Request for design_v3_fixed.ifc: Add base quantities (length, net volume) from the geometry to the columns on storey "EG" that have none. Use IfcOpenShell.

First a look at what the model holds.

```python
import ifcopenshell
import ifcopenshell.util.element
import ifcopenshell.util.unit

model = ifcopenshell.open("design_v3_fixed.ifc")
print(model.schema)
for unit_type in ("LENGTHUNIT", "AREAUNIT", "VOLUMEUNIT"):
    print(unit_type, ifcopenshell.util.unit.calculate_unit_scale(model, unit_type))
storey = next(s for s in model.by_type("IfcBuildingStorey") if s.Name == "EG")
columns = [e for e in ifcopenshell.util.element.get_decomposition(storey) if e.is_a("IfcColumn")]
for e in sorted(columns, key=lambda e: e.id()):
    print(e.id(), e.is_a(), e.Name, list(ifcopenshell.util.element.get_psets(e, qtos_only=True)), sep=" | ")
```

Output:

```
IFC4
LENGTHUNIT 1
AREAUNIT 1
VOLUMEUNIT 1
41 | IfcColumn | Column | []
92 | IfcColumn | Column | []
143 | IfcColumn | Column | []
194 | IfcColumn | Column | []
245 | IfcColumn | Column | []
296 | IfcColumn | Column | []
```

```python
import ifcopenshell
import ifcopenshell.api.pset
import ifcopenshell.geom
import ifcopenshell.util.element
import ifcopenshell.util.shape
import ifcopenshell.util.unit

model = ifcopenshell.open("design_v3_fixed.ifc")
unit_scale = ifcopenshell.util.unit.calculate_unit_scale(model)
volume_scale = ifcopenshell.util.unit.calculate_unit_scale(model, "VOLUMEUNIT")
settings = ifcopenshell.geom.settings()

storey = next(s for s in model.by_type("IfcBuildingStorey") if s.Name == "EG")
columns = [e for e in ifcopenshell.util.element.get_decomposition(storey) if e.is_a("IfcColumn")]

for e in sorted(columns, key=lambda e: e.id()):
    if ifcopenshell.util.element.get_psets(e, qtos_only=True, should_inherit=False):
        continue
    # Geometry comes back in metres, in the element's own axes.
    shape = ifcopenshell.geom.create_shape(settings, e)
    values = {
        "Length": ifcopenshell.util.shape.get_z(shape.geometry) / unit_scale,
        "NetVolume": ifcopenshell.util.shape.get_volume(shape.geometry) / volume_scale,
    }
    qto = ifcopenshell.api.pset.add_qto(model, product=e, name="Qto_ColumnBaseQuantities")
    ifcopenshell.api.pset.edit_qto(model, qto=qto, properties=values)
    print(e.id(), {k: round(v, 3) for k, v in values.items()})

model.write("design_v3_fixed_v2.ifc")
```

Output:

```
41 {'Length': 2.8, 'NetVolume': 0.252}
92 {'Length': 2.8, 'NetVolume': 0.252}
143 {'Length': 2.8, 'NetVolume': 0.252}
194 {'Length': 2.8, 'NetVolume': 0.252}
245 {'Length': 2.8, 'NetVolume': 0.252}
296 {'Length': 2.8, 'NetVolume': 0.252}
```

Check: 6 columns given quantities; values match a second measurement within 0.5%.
